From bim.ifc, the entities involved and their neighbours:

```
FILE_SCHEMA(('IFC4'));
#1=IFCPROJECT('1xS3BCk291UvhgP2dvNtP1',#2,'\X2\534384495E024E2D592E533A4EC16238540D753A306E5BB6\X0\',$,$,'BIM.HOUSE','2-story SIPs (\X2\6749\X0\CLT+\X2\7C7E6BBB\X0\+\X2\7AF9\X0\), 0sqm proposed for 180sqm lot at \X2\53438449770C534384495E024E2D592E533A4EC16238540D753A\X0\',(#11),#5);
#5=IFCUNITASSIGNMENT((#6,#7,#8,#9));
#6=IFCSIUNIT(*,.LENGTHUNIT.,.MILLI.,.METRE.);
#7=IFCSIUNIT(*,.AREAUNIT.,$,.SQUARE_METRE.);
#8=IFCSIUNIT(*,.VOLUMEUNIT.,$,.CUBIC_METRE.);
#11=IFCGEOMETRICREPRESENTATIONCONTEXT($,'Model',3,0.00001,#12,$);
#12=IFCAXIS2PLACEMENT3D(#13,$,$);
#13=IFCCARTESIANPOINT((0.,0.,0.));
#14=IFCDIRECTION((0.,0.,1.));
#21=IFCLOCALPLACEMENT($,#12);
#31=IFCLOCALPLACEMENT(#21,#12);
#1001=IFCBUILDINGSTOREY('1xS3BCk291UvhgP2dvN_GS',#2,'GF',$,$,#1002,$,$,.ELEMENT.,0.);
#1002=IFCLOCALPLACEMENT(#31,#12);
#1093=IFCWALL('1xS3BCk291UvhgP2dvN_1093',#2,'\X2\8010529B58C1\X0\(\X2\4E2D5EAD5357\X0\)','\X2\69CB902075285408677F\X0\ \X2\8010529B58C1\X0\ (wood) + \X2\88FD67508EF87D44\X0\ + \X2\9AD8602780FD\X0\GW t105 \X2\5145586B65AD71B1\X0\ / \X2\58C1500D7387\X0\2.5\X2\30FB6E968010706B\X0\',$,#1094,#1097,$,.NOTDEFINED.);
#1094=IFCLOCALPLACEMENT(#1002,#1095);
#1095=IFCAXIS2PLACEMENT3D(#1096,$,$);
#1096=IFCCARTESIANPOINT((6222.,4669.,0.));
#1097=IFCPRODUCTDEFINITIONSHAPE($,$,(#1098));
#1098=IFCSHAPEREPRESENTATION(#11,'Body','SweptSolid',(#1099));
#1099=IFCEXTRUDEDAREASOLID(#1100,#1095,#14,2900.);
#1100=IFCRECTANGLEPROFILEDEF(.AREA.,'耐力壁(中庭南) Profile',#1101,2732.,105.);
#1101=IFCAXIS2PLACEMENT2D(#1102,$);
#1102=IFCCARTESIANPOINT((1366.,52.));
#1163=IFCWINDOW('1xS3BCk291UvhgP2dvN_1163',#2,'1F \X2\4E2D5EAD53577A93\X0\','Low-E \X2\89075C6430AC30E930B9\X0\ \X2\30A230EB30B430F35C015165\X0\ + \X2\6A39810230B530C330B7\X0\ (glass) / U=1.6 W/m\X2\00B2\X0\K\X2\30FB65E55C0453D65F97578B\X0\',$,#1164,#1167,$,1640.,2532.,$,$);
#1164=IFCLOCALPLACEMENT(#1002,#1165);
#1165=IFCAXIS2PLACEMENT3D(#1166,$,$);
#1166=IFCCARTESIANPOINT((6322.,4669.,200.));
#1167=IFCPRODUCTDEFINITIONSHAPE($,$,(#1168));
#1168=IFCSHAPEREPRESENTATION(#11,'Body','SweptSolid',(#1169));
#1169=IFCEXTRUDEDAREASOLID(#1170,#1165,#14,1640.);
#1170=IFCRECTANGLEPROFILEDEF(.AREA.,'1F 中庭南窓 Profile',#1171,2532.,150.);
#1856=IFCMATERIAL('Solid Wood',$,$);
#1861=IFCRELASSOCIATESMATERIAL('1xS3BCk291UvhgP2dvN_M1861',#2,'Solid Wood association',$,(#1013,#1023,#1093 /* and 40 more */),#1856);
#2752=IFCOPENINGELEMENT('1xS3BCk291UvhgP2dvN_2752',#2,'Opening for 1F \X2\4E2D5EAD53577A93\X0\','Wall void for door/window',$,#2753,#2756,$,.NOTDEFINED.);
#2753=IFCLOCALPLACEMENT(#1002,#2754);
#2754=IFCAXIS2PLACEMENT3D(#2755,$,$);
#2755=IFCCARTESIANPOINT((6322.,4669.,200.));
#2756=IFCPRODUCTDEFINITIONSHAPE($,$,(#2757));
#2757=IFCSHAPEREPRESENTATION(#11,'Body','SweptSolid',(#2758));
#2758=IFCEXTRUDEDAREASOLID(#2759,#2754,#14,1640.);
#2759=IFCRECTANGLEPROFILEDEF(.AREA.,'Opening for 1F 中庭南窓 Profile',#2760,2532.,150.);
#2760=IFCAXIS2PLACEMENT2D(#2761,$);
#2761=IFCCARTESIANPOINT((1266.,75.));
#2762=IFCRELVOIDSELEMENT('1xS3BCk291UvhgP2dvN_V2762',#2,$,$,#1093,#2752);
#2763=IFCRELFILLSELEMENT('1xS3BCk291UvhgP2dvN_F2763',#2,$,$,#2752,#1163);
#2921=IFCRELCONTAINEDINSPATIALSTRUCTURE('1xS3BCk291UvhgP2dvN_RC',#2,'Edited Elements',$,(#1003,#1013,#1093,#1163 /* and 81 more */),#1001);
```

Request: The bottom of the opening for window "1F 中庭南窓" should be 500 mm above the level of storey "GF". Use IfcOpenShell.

```python
import numpy as np
import ifcopenshell
import ifcopenshell.api.geometry
import ifcopenshell.geom
import ifcopenshell.util.element
import ifcopenshell.util.placement
import ifcopenshell.util.shape
import ifcopenshell.util.unit

model = ifcopenshell.open("bim.ifc")
unit_scale = ifcopenshell.util.unit.calculate_unit_scale(model)

window = model.by_guid("1xS3BCk291UvhgP2dvN_1163")
opening = window.FillsVoids[0].RelatingOpeningElement
storey = ifcopenshell.util.element.get_container(window, ifc_class="IfcBuildingStorey")
level = ifcopenshell.util.placement.get_local_placement(storey.ObjectPlacement)[2, 3]

# The opening's origin need not be at the sill, so measure its lowest point.
shape = ifcopenshell.geom.create_shape(ifcopenshell.geom.settings(), opening)
bottom = ifcopenshell.util.shape.get_shape_bottom_elevation(shape, shape.geometry) / unit_scale
dz = level + 500.0 - bottom

shift = np.array([0.0, 0.0, dz])
# The window is not placed relative to its opening, so move both.
for product in (opening, window):
    matrix = ifcopenshell.util.placement.get_local_placement(product.ObjectPlacement)
    matrix[:3, 3] += shift
    ifcopenshell.api.geometry.edit_object_placement(model, product=product, matrix=matrix, is_si=False)

print(f"moved by {dz * unit_scale:+.3f} m")

model.write("bim-out.ifc")
```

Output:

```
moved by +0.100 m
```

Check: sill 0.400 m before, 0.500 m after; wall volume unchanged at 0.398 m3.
